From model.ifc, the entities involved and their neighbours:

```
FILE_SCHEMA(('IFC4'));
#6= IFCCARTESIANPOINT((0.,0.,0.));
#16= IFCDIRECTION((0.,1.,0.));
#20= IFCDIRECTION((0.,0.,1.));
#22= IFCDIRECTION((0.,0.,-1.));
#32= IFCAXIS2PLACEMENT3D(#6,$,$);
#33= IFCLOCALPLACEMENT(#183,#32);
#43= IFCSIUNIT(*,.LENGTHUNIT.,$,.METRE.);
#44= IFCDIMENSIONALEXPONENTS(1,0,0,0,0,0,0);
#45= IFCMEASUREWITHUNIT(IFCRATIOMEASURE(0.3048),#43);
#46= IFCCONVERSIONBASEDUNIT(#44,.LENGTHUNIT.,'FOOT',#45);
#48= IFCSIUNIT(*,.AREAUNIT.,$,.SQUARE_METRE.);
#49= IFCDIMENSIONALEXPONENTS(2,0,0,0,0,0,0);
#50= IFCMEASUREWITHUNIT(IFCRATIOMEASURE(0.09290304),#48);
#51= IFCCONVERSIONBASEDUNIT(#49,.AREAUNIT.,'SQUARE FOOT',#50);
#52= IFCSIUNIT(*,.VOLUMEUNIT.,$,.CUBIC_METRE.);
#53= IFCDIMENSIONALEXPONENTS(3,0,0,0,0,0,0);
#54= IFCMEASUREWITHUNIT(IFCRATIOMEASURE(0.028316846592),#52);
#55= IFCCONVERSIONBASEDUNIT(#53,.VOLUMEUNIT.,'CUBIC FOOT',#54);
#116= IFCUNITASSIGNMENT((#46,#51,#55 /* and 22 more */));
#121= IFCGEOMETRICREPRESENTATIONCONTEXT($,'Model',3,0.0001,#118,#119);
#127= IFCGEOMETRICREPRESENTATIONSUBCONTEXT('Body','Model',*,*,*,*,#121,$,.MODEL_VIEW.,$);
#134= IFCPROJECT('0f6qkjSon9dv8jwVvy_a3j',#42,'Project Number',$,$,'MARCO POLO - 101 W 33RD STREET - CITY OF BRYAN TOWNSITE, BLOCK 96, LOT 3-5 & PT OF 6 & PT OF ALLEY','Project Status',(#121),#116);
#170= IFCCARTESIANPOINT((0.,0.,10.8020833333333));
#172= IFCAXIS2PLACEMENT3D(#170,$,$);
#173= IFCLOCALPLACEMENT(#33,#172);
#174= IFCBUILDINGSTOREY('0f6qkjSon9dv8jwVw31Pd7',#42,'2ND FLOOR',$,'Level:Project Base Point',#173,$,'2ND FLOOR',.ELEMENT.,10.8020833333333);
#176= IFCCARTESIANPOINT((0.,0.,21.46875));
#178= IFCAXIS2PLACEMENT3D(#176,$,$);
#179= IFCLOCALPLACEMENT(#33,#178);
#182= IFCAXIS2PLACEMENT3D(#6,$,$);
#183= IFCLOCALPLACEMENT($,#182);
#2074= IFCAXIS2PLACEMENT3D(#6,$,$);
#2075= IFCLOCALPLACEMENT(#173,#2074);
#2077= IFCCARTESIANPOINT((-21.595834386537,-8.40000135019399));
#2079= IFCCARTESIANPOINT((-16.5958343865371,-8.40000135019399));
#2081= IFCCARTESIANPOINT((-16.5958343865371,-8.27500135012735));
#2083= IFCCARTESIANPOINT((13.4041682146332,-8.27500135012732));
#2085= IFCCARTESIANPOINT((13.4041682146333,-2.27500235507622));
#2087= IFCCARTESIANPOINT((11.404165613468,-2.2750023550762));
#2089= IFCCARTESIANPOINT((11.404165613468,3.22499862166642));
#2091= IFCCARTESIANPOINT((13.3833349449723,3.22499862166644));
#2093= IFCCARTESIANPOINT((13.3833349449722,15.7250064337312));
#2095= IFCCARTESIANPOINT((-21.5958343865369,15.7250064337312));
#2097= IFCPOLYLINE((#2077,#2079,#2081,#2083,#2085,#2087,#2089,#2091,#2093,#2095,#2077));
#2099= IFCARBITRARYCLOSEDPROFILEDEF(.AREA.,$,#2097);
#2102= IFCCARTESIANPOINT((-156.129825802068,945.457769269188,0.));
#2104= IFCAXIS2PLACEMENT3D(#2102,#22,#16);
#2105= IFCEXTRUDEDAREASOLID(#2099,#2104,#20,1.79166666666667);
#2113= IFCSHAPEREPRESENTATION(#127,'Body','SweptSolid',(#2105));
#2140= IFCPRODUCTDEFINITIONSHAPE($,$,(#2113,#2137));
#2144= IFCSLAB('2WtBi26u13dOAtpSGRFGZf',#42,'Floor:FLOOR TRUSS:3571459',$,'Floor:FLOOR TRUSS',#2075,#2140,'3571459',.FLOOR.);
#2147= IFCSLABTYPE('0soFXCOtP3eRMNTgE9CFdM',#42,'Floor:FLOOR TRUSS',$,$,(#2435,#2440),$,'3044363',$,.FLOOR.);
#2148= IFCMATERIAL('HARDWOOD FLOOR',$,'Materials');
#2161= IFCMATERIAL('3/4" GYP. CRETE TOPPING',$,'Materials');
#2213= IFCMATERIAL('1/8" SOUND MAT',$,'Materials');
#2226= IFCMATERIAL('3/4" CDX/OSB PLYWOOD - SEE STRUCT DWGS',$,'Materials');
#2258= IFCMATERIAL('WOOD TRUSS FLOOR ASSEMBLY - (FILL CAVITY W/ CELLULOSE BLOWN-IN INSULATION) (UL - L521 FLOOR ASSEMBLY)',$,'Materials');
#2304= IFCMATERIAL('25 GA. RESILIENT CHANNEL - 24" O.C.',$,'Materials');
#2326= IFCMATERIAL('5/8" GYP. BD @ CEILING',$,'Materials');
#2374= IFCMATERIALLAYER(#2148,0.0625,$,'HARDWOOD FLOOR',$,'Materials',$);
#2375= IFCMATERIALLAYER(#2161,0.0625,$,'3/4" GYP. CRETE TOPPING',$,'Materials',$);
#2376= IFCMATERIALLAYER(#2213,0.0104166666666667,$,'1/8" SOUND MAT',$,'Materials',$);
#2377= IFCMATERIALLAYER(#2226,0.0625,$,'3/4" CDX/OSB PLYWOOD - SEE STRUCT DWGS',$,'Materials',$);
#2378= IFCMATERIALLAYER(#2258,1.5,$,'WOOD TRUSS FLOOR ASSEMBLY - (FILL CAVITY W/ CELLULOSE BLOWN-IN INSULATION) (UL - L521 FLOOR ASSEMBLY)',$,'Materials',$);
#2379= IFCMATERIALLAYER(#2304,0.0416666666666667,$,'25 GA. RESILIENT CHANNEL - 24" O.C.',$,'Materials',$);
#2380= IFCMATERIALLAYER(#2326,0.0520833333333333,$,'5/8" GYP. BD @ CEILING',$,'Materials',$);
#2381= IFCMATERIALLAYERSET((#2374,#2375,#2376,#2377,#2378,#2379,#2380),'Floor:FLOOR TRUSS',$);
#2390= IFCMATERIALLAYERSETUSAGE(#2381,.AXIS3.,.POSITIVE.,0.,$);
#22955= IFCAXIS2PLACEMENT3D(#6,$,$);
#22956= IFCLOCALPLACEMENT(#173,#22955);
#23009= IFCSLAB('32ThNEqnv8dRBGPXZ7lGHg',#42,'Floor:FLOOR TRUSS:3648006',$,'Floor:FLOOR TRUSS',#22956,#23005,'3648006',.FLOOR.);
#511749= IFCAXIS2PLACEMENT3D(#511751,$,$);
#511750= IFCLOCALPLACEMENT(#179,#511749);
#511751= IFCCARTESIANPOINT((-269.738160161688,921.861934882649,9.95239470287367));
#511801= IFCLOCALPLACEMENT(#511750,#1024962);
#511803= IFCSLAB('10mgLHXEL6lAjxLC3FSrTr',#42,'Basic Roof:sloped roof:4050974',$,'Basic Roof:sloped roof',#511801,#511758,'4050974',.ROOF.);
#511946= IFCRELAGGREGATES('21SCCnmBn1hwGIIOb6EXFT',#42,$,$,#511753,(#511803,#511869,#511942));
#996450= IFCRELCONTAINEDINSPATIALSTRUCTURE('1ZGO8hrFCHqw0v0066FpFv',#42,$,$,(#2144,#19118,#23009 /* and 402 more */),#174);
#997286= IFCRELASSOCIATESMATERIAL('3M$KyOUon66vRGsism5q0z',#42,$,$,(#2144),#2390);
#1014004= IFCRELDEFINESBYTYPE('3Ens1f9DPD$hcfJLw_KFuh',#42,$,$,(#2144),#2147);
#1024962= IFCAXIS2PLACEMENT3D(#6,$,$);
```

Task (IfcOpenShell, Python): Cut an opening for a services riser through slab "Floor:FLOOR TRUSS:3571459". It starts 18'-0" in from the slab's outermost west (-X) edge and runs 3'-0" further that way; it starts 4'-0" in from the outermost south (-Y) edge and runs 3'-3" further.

```python
import numpy as np
import ifcopenshell
import ifcopenshell.api.feature
import ifcopenshell.api.geometry
import ifcopenshell.api.root
import ifcopenshell.geom
import ifcopenshell.util.placement
import ifcopenshell.util.representation
import ifcopenshell.util.shape
import ifcopenshell.util.unit

model = ifcopenshell.open("model.ifc")
unit_scale = ifcopenshell.util.unit.calculate_unit_scale(model)
settings = ifcopenshell.geom.settings()


def volume(element):
    """Net volume in cubic metres, openings subtracted."""
    shape = ifcopenshell.geom.create_shape(settings, element)
    return ifcopenshell.util.shape.get_volume(shape.geometry)


slab = model.by_id(2144)
before = volume(slab)

# Extent in the slab's own axes, in metres. The edges named are its -X and -Y sides.
slab_shape = ifcopenshell.geom.create_shape(settings, slab)
vertices = ifcopenshell.util.shape.get_vertices(slab_shape.geometry)
x_min, y_min, bottom = vertices.min(axis=0)
top = vertices[:, 2].max()

opening = ifcopenshell.api.root.create_entity(model, ifc_class="IfcOpeningElement", name="Services riser opening", predefined_type="OPENING")
context = ifcopenshell.util.representation.get_context(model, "Model", "Body", "MODEL_VIEW")
width, depth = 0.9144, 0.9906
outline = [(0.0, 0.0), (width, 0.0), (width, depth), (0.0, depth), (0.0, 0.0)]
# Overshoot both faces by 50 mm so the cut is clean.
shape = ifcopenshell.api.geometry.add_slab_representation(
    model, context=context, depth=top - bottom + 0.1, polyline=outline
)
ifcopenshell.api.geometry.assign_representation(model, product=opening, representation=shape)

matrix = ifcopenshell.util.placement.get_local_placement(slab.ObjectPlacement)
matrix[:, 3] = matrix @ np.append(np.array([x_min + 5.4864, y_min + 1.2192, bottom - 0.05]) / unit_scale, 1.0)
ifcopenshell.api.geometry.edit_object_placement(model, product=opening, matrix=matrix, is_si=False)
ifcopenshell.api.feature.add_feature(model, feature=opening, element=slab)

after = volume(slab)

print(f"slab volume {before:.3f} -> {after:.3f} m3")

model.write("model_updated.ifc")
```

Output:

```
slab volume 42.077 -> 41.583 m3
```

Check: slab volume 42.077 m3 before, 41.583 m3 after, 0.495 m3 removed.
